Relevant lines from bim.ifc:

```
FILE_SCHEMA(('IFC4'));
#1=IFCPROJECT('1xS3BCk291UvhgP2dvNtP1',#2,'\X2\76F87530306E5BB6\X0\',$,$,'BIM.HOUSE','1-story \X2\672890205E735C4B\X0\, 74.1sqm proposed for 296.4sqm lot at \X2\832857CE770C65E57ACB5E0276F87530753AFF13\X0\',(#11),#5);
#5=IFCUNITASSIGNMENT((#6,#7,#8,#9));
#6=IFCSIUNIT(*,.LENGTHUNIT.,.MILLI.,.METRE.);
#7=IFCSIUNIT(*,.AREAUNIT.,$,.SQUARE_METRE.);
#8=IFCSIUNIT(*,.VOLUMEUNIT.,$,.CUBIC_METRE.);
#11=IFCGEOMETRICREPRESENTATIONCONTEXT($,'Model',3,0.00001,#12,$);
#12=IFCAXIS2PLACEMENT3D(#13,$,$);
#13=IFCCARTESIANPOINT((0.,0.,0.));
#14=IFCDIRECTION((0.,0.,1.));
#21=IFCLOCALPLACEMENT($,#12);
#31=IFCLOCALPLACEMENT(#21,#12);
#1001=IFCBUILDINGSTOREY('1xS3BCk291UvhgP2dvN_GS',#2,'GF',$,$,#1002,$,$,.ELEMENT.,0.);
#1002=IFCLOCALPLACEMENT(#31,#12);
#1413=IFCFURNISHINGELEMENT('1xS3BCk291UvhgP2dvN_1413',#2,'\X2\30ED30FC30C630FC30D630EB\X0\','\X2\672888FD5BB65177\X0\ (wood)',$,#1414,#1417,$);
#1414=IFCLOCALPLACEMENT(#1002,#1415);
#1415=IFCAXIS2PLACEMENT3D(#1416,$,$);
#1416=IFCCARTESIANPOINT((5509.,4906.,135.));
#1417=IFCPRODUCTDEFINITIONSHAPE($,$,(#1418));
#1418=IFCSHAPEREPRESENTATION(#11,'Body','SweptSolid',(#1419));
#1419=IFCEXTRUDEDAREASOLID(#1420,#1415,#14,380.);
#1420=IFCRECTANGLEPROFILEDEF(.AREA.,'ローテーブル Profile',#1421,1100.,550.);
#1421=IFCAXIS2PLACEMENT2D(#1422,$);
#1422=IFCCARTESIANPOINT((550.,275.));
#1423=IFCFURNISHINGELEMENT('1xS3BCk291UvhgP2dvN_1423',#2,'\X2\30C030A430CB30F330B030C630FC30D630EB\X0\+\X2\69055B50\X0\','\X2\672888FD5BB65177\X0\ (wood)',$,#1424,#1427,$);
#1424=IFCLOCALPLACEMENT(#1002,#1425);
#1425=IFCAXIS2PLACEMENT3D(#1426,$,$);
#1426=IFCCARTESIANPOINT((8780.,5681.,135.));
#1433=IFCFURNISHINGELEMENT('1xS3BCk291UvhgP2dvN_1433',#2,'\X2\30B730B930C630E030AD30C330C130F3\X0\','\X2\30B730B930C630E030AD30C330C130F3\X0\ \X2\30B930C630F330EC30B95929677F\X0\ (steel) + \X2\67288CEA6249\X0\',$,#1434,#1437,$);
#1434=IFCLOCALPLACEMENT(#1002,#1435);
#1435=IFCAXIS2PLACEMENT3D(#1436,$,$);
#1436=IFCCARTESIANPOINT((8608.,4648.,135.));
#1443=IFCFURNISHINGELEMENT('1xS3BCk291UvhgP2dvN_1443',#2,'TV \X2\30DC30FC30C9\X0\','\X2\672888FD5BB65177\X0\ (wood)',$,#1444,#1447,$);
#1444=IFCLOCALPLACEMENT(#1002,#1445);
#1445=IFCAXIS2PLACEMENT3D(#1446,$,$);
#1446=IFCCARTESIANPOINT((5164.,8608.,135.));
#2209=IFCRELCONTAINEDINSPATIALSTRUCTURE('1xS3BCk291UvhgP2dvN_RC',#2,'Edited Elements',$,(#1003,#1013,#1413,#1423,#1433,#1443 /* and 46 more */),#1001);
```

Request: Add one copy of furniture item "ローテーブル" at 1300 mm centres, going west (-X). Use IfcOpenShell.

```python
import numpy as np
import ifcopenshell
import ifcopenshell.api.geometry
import ifcopenshell.api.root
import ifcopenshell.util.element
import ifcopenshell.util.placement

model = ifcopenshell.open("bim.ifc")


def reuse_history(source, copy):
    """copy_class also copies each property set's owner history, people and application; keep the originals."""
    for rel in copy.IsDefinedBy:
        if rel.is_a("IfcRelDefinesByProperties") and (history := rel.RelatingPropertyDefinition.OwnerHistory):
            rel.RelatingPropertyDefinition.OwnerHistory = source.OwnerHistory
            ifcopenshell.util.element.remove_deep2(model, history)


source = model.by_guid("1xS3BCk291UvhgP2dvN_1413")
base = ifcopenshell.util.placement.get_local_placement(source.ObjectPlacement)
step = np.array([-1.0, 0.0, 0.0]) * 1300.0

for i in range(1, 2):
    copy = ifcopenshell.api.root.copy_class(model, product=source)
    copy.Representation = ifcopenshell.util.element.copy_deep(
        model, source.Representation, exclude=["IfcGeometricRepresentationContext", "IfcRepresentationMap"]
    )
    reuse_history(source, copy)
    matrix = base.copy()
    matrix[:3, 3] += i * step
    print("added at", matrix[:3, 3].round(3) + 0.0)
    ifcopenshell.api.geometry.edit_object_placement(model, product=copy, matrix=matrix, is_si=False)

model.write("bim_rev.ifc")
```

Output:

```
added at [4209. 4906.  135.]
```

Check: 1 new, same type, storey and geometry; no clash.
